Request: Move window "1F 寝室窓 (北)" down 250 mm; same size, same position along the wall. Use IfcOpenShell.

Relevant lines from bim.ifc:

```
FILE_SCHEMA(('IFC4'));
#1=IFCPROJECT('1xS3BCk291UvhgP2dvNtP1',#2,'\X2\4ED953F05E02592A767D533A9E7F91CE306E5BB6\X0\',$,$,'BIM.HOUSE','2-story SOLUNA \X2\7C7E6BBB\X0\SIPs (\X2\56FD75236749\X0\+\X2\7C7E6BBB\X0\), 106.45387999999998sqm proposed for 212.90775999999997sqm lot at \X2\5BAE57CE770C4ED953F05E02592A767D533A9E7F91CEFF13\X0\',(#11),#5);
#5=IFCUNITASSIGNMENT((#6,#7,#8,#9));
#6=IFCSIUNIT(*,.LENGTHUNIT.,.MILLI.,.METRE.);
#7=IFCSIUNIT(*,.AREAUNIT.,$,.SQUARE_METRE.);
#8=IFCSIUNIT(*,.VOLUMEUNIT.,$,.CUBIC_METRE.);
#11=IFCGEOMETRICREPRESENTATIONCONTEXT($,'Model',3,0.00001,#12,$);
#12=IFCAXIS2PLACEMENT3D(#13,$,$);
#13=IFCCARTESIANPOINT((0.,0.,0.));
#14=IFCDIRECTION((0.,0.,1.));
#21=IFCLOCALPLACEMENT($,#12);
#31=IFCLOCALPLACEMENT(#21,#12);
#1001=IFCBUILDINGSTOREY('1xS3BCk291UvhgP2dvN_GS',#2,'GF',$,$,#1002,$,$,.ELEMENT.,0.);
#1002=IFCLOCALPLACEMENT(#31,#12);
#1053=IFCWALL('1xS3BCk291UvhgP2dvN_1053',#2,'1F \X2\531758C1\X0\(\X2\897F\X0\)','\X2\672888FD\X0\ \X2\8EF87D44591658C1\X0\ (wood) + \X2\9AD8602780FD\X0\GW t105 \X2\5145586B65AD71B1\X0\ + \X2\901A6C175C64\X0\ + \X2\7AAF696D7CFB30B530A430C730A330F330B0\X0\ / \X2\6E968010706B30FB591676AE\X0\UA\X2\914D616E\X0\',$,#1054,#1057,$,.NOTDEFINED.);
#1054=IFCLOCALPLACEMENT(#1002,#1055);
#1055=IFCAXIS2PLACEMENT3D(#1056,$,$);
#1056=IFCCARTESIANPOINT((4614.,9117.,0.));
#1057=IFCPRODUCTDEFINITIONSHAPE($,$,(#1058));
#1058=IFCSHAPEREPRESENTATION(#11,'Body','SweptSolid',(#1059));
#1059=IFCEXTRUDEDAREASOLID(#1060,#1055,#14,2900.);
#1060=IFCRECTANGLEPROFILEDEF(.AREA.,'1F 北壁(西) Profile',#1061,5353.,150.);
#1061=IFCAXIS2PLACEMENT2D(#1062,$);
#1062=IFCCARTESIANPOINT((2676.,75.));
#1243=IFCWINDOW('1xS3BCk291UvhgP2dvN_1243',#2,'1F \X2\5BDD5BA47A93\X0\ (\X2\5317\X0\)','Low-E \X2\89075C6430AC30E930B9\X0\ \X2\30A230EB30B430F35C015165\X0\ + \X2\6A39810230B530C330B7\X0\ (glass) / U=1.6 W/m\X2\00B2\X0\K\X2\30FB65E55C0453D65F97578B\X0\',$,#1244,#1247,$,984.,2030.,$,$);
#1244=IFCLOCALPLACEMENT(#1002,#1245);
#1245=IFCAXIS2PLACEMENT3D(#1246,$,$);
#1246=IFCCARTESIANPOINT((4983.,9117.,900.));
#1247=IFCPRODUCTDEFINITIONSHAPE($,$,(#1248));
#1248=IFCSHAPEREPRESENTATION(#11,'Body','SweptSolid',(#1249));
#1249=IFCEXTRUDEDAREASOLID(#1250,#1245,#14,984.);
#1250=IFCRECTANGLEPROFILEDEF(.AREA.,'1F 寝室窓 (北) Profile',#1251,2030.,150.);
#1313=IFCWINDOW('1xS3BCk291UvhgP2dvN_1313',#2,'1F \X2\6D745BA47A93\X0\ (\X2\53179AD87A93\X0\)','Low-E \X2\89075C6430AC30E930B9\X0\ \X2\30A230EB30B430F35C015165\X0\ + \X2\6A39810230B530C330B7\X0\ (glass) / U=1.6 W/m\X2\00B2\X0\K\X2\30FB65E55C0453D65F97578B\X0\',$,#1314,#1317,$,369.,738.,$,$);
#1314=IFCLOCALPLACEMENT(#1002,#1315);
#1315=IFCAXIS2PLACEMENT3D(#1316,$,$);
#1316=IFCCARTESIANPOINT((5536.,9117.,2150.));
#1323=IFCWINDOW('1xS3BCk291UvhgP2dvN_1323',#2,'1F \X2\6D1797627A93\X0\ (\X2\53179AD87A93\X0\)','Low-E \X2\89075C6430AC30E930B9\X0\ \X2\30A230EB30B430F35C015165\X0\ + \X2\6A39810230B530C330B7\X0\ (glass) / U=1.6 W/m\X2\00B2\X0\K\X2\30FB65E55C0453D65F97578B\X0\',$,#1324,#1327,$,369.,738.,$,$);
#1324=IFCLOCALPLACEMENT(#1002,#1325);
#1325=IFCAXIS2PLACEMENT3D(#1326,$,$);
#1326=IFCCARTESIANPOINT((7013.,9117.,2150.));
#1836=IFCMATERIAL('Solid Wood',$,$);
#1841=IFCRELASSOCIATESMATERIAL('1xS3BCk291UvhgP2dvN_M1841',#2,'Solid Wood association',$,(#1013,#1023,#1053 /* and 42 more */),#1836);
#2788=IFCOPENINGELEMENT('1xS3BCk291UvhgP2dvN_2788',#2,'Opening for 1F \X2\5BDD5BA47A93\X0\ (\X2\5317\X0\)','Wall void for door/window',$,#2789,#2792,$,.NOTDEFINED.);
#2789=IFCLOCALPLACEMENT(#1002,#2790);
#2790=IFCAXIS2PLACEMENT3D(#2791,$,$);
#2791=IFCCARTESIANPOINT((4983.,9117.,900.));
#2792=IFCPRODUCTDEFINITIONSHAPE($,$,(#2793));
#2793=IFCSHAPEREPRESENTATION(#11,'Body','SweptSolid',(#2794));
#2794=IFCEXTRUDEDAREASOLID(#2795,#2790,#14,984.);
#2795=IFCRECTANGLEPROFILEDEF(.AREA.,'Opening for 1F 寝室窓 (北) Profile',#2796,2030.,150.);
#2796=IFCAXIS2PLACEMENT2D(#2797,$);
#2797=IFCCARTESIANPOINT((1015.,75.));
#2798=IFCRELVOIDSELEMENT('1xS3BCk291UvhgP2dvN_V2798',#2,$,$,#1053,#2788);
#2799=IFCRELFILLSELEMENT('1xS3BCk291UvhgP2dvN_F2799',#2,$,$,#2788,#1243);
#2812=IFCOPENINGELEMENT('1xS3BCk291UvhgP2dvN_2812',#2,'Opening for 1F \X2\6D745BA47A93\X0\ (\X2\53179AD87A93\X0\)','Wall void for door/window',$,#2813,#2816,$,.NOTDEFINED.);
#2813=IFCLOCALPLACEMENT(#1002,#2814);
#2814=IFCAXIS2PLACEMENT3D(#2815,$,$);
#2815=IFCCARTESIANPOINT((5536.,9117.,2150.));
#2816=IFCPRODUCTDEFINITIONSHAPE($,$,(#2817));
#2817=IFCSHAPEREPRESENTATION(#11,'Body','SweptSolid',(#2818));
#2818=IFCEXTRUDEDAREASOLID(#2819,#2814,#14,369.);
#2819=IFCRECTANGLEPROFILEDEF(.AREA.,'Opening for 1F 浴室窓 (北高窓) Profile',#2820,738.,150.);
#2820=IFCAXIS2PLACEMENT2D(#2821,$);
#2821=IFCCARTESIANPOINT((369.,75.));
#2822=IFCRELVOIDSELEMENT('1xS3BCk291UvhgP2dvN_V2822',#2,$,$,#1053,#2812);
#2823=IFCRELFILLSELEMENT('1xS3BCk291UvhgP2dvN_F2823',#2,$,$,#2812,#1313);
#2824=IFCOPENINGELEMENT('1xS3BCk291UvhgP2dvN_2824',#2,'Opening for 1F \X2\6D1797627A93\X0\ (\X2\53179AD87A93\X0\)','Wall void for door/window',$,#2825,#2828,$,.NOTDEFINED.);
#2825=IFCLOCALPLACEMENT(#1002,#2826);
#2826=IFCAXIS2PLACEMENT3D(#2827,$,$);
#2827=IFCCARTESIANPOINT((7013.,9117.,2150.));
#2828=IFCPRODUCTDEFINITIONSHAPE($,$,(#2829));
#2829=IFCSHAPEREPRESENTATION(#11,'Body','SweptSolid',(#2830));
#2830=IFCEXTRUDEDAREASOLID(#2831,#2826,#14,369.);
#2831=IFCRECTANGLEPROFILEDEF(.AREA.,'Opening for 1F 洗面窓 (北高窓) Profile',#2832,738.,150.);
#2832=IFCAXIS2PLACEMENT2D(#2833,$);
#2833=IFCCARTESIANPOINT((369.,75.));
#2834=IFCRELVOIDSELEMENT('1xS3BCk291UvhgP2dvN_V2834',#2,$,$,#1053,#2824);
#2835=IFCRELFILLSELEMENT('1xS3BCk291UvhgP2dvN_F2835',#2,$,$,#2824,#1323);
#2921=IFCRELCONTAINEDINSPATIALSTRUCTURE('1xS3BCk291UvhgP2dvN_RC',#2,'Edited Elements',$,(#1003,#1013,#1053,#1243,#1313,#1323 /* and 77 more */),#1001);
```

```python
import numpy as np
import ifcopenshell
import ifcopenshell.api.geometry
import ifcopenshell.util.placement
import ifcopenshell.util.unit

model = ifcopenshell.open("bim.ifc")
unit_scale = ifcopenshell.util.unit.calculate_unit_scale(model)

window = model.by_guid("1xS3BCk291UvhgP2dvN_1243")
opening = window.FillsVoids[0].RelatingOpeningElement
dz = -250.0

shift = np.array([0.0, 0.0, dz])
# The window is not placed relative to its opening, so move both.
for product in (opening, window):
    matrix = ifcopenshell.util.placement.get_local_placement(product.ObjectPlacement)
    matrix[:3, 3] += shift
    ifcopenshell.api.geometry.edit_object_placement(model, product=product, matrix=matrix, is_si=False)

print(f"moved by {dz * unit_scale:+.3f} m")

model.write("bim-out.ifc")
```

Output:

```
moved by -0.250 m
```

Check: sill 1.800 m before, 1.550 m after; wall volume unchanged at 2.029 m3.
